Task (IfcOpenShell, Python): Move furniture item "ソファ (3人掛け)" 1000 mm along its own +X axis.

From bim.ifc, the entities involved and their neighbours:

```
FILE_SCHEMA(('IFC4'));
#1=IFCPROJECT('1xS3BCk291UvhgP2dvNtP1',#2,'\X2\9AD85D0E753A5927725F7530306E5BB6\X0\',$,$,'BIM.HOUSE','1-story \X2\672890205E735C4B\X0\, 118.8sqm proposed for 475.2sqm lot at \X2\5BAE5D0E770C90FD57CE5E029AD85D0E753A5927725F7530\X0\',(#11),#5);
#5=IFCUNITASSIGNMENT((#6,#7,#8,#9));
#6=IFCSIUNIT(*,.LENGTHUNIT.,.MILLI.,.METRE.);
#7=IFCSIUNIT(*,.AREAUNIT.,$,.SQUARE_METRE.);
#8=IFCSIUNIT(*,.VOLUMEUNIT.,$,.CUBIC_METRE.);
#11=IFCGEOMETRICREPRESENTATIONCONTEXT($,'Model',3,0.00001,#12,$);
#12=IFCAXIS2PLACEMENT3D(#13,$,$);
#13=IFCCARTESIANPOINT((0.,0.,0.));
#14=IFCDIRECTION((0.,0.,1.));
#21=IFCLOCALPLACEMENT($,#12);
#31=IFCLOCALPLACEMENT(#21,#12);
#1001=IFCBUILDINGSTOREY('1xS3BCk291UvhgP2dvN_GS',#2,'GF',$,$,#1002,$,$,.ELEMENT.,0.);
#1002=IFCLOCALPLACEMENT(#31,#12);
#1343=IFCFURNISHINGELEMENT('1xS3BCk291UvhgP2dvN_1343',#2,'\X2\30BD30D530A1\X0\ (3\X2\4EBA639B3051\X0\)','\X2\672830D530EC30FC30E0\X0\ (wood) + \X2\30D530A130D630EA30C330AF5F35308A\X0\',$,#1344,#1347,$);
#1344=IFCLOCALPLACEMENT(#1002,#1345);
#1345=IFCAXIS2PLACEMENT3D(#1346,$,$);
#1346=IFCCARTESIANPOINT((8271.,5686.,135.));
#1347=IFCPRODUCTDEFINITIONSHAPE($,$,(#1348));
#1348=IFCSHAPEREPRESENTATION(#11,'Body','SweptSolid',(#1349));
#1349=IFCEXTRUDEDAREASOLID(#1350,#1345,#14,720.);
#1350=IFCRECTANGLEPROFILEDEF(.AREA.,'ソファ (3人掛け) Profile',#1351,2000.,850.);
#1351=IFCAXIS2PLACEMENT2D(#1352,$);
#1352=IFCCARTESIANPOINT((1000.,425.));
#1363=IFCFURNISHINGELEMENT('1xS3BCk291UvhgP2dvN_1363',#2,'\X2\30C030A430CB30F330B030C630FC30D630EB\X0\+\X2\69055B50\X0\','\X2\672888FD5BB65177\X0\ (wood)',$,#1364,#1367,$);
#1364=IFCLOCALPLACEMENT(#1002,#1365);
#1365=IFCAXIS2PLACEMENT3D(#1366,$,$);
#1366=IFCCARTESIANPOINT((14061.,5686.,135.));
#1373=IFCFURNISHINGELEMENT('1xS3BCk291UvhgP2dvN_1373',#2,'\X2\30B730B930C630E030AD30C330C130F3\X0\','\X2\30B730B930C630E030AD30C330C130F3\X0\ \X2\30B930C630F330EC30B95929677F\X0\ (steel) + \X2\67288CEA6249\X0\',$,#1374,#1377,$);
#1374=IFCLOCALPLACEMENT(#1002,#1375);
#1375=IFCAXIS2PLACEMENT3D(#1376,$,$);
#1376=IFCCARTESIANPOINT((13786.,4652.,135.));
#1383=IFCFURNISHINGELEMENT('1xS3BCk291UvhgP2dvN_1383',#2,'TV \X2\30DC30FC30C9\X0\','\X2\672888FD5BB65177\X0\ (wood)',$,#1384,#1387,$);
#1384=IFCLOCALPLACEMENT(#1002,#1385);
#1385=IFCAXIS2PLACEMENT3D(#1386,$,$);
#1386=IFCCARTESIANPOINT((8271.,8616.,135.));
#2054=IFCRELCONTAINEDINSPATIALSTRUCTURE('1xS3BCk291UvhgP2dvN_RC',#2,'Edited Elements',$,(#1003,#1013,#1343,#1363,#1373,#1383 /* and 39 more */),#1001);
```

```python
import ifcopenshell
import ifcopenshell.api.geometry
import ifcopenshell.util.placement

model = ifcopenshell.open("bim.ifc")

item = model.by_guid("1xS3BCk291UvhgP2dvN_1343")
matrix = ifcopenshell.util.placement.get_local_placement(item.ObjectPlacement)
matrix[:3, 3] += matrix[:3, 0] * 1000.0
ifcopenshell.api.geometry.edit_object_placement(model, product=item, matrix=matrix, is_si=False)

print(ifcopenshell.util.placement.get_local_placement(item.ObjectPlacement).round(3) + 0.0)

model.write("bim_v2.ifc")
```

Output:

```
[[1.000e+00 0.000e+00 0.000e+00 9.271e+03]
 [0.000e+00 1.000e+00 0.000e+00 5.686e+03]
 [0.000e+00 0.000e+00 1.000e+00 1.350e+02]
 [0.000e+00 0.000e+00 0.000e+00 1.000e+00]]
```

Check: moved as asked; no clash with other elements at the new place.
